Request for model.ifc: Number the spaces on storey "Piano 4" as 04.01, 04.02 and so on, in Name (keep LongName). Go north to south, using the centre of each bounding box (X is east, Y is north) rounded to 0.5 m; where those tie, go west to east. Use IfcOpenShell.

First a look at what the model holds.

```python
import ifcopenshell
import ifcopenshell.util.element
import ifcopenshell.util.placement

model = ifcopenshell.open("model.ifc")
print(model.schema)
storey = next(s for s in model.by_type("IfcBuildingStorey") if s.Name == "Piano 4")
spaces = [e for e in ifcopenshell.util.element.get_decomposition(storey) if e.is_a("IfcSpace")]
for e in sorted(spaces, key=lambda e: e.id()):
    origin = ifcopenshell.util.placement.get_local_placement(e.ObjectPlacement)[:3, 3]
    print(e.id(), e.Name, e.LongName, origin.round(2) + 0.0, sep=" | ")
```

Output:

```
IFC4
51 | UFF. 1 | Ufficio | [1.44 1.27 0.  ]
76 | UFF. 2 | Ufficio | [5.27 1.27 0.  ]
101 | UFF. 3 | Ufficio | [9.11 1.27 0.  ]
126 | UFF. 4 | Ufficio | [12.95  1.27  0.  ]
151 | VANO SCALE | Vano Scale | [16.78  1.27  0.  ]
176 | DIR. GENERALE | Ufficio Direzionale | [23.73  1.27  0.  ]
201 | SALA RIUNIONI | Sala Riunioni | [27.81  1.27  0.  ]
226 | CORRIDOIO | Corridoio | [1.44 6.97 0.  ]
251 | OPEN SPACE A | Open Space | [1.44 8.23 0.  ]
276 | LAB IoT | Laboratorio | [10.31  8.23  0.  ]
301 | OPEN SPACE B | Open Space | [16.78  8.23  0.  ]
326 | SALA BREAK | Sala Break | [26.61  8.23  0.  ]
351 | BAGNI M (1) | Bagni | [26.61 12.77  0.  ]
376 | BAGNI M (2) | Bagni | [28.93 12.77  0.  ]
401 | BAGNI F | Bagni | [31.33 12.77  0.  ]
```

```python
import ifcopenshell
import ifcopenshell.geom
import ifcopenshell.util.element
import ifcopenshell.util.shape

model = ifcopenshell.open("model.ifc")
settings = ifcopenshell.geom.settings()
settings.set("use-world-coords", True)


def centre(element):
    shape = ifcopenshell.geom.create_shape(settings, element)
    return ifcopenshell.util.shape.get_bbox_centroid(shape.geometry)


storey = next(s for s in model.by_type("IfcBuildingStorey") if s.Name == "Piano 4")
spaces = [e for e in ifcopenshell.util.element.get_decomposition(storey) if e.is_a("IfcSpace")]

# Insertion points can sit at a corner or the storey origin, so sort by the geometry (in metres).
centres = {e: centre(e) for e in spaces}
spaces.sort(key=lambda e: (-round(centres[e][1] / 0.5), centres[e][0]))

for i, e in enumerate(spaces, start=1):
    number = f"04.{i:02d}"
    e.Name = number
    print(e.id(), number)

model.write("model_updated.ifc")
```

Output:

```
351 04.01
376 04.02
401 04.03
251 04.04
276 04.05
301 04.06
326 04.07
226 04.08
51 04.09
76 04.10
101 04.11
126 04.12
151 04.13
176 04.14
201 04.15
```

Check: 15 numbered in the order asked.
